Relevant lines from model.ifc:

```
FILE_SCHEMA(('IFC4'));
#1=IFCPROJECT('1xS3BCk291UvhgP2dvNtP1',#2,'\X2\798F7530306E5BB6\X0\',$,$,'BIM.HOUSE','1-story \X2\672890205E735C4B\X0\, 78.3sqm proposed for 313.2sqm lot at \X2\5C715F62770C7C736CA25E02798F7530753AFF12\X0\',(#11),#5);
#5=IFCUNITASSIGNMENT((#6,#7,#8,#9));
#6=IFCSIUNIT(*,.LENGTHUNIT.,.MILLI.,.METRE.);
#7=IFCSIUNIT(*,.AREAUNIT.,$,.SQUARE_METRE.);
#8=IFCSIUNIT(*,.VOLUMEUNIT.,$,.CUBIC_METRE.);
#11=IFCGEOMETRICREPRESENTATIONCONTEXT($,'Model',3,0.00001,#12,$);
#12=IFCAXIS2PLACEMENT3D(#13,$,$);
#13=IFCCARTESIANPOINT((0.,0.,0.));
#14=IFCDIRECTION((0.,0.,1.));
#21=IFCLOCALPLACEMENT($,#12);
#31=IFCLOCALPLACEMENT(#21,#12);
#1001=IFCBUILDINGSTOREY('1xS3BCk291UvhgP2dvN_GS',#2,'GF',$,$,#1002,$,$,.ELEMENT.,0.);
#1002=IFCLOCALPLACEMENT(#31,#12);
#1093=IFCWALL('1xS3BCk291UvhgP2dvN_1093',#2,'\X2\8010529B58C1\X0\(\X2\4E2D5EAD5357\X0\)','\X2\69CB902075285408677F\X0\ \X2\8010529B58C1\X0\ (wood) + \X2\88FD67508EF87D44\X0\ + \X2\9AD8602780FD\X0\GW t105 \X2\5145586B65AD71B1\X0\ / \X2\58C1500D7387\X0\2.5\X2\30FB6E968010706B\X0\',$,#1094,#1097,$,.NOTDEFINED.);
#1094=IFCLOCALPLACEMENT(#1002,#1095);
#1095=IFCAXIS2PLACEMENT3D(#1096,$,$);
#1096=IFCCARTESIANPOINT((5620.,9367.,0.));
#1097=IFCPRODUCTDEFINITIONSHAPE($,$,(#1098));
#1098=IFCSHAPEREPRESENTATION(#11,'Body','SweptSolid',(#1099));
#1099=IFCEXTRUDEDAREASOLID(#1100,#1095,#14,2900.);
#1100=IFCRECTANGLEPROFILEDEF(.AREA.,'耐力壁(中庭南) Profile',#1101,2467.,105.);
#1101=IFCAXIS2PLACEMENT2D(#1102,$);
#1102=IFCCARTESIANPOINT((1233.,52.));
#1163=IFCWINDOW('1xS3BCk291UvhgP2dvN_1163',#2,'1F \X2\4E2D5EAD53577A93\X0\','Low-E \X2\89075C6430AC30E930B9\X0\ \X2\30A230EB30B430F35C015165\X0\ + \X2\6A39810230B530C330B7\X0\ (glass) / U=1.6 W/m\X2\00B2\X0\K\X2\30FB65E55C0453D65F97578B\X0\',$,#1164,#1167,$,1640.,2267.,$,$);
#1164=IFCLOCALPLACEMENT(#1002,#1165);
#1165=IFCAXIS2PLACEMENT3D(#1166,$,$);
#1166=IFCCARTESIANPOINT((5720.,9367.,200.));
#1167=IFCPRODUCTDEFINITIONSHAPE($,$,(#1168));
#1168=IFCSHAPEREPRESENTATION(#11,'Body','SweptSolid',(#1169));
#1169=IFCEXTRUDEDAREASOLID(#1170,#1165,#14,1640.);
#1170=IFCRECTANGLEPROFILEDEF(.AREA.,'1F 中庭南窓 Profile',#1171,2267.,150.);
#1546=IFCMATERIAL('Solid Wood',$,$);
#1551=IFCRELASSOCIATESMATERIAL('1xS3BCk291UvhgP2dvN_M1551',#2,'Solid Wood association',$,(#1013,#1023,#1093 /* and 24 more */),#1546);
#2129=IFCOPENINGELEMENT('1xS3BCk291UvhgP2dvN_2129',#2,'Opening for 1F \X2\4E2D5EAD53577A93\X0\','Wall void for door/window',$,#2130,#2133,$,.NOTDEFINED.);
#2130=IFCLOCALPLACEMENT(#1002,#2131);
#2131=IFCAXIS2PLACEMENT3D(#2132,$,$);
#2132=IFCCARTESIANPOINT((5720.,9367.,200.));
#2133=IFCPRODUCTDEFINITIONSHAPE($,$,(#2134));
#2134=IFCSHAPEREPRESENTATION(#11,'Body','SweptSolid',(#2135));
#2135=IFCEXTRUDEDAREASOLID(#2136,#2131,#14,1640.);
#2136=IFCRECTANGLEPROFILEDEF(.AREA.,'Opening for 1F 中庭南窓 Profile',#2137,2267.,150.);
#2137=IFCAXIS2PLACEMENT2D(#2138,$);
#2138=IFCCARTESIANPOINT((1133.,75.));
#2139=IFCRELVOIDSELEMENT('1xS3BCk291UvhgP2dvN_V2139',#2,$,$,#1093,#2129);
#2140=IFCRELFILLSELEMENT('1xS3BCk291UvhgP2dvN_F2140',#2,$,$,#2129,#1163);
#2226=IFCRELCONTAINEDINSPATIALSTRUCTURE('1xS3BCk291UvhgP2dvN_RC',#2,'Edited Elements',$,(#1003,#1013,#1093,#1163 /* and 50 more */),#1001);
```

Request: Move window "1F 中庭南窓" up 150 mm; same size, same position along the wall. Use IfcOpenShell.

```python
import numpy as np
import ifcopenshell
import ifcopenshell.api.geometry
import ifcopenshell.util.placement
import ifcopenshell.util.unit

model = ifcopenshell.open("model.ifc")
unit_scale = ifcopenshell.util.unit.calculate_unit_scale(model)

window = model.by_guid("1xS3BCk291UvhgP2dvN_1163")
opening = window.FillsVoids[0].RelatingOpeningElement
dz = 150.0

shift = np.array([0.0, 0.0, dz])
# The window is not placed relative to its opening, so move both.
for product in (opening, window):
    matrix = ifcopenshell.util.placement.get_local_placement(product.ObjectPlacement)
    matrix[:3, 3] += shift
    ifcopenshell.api.geometry.edit_object_placement(model, product=product, matrix=matrix, is_si=False)

print(f"moved by {dz * unit_scale:+.3f} m")

model.write("model_updated.ifc")
```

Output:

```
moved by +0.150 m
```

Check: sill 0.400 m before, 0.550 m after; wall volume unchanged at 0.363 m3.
